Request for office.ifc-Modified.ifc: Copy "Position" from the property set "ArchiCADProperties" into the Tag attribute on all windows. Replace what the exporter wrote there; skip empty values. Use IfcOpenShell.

First a look at what the model holds.

```python
import ifcopenshell
import ifcopenshell.util.element

model = ifcopenshell.open("office.ifc-Modified.ifc")
print(model.schema)
windows = model.by_type("IfcWindow")
print(len(windows), "windows")
for e in windows[:8]:
    source = ifcopenshell.util.element.get_pset(e, "ArchiCADProperties", "Position")
    target = e.Tag
    print(e.id(), repr(source), repr(target), sep=" | ")
```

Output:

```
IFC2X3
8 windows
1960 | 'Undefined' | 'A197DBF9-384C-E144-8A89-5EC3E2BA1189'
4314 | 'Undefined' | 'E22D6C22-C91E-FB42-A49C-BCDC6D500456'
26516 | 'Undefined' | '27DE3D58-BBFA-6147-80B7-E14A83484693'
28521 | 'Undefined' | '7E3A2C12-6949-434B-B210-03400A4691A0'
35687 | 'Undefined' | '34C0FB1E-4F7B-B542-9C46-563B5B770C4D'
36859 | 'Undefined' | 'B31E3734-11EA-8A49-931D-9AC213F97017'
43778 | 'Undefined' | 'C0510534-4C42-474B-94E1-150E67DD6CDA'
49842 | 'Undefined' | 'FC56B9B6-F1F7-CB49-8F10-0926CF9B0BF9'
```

```python
import ifcopenshell
import ifcopenshell.util.element

model = ifcopenshell.open("office.ifc-Modified.ifc")

count = 0
for e in model.by_type("IfcWindow"):
    value = ifcopenshell.util.element.get_pset(e, "ArchiCADProperties", "Position")
    current = e.Tag
    if not value or not value.strip() or current == value:
        continue
    e.Tag = value
    count += 1

print(count, "windows updated")

model.write("office.ifc-Modified_edited.ifc")
```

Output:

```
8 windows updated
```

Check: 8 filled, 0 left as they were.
